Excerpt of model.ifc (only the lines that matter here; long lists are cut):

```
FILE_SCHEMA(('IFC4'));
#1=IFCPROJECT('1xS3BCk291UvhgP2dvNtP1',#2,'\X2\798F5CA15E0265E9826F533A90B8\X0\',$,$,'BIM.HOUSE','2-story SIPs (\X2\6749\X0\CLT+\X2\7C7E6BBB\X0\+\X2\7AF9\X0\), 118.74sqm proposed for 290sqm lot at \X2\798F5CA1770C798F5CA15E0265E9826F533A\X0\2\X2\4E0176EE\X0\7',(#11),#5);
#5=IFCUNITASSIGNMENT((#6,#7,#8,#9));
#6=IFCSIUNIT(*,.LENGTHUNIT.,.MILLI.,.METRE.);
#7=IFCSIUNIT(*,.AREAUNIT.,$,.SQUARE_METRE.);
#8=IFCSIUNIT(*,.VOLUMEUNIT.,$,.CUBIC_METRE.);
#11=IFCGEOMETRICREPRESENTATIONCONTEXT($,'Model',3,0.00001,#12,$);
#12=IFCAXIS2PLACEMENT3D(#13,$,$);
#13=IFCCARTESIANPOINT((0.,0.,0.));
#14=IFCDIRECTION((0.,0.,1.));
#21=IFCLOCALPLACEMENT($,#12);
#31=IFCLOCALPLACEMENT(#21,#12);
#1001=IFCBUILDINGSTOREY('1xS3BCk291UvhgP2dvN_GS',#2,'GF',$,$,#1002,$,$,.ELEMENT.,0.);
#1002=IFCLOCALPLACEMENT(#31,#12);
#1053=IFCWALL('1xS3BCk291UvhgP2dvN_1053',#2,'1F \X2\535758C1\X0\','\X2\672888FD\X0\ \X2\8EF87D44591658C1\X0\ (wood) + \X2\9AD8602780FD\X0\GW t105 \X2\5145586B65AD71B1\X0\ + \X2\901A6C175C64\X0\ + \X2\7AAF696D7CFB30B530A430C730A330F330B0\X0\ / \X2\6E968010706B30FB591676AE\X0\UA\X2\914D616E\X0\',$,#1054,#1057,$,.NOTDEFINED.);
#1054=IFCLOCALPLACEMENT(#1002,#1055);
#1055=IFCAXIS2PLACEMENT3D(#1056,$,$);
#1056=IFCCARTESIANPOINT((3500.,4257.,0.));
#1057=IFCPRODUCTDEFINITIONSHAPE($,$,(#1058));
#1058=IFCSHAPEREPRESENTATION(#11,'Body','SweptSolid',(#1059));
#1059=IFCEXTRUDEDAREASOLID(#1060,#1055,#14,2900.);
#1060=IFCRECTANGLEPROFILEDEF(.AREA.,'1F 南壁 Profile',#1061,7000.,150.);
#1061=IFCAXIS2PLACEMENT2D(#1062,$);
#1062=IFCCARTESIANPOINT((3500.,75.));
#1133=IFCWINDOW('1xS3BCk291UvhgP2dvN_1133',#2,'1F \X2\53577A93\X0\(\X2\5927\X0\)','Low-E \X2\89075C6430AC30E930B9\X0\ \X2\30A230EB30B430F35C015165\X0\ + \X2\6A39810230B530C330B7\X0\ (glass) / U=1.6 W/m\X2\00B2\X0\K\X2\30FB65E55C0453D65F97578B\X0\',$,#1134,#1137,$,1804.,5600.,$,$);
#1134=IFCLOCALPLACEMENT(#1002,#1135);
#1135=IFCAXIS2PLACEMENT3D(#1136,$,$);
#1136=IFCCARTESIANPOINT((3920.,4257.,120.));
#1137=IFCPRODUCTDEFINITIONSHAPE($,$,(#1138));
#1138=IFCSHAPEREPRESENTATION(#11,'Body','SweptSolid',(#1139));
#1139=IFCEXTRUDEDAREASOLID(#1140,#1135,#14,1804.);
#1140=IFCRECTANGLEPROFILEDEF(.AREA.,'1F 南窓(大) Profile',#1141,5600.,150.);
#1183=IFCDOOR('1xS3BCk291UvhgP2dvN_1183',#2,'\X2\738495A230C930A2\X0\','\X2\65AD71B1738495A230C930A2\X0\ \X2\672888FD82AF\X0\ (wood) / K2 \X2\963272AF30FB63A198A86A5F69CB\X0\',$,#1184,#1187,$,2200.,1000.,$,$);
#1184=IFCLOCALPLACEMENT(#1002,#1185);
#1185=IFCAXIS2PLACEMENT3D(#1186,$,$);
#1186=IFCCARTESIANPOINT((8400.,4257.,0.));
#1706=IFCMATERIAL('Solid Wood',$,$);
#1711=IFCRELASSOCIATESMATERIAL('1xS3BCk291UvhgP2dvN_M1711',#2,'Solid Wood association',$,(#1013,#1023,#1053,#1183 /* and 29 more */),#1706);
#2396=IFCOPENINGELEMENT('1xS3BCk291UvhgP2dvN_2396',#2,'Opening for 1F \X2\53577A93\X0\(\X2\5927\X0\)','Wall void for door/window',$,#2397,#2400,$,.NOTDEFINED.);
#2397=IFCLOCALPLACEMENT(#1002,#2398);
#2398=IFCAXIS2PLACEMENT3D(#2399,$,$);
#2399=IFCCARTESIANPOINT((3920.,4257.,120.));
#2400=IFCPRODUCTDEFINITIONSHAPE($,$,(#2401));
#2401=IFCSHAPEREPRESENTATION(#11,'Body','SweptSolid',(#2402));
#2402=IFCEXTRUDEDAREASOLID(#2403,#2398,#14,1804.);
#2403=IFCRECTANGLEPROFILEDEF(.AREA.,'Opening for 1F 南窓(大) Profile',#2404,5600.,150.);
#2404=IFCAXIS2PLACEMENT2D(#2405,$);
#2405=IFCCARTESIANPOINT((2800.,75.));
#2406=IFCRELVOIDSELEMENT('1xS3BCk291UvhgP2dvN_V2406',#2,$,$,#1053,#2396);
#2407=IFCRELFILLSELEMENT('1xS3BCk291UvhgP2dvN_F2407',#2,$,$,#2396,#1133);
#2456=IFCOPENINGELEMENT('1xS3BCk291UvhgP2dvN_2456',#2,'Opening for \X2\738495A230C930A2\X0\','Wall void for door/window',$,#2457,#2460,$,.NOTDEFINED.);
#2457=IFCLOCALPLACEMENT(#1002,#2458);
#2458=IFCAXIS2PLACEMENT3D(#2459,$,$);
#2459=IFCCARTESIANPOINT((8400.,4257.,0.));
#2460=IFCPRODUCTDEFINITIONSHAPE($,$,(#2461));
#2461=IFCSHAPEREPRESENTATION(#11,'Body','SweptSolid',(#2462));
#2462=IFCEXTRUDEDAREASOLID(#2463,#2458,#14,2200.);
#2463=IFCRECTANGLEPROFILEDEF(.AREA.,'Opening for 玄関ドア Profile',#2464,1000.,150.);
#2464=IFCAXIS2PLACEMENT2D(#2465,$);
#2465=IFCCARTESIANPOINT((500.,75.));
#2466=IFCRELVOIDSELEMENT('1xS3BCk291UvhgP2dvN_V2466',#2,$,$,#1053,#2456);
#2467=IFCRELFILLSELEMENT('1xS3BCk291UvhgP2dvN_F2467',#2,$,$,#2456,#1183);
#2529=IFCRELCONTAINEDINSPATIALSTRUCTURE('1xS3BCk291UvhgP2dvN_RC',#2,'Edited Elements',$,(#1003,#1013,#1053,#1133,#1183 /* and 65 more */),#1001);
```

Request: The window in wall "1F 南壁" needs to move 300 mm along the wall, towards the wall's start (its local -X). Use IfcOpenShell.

```python
import ifcopenshell
import ifcopenshell.api.geometry
import ifcopenshell.util.placement
import ifcopenshell.util.unit

model = ifcopenshell.open("model.ifc")
unit_scale = ifcopenshell.util.unit.calculate_unit_scale(model)

window = model.by_guid("1xS3BCk291UvhgP2dvN_1133")
opening = window.FillsVoids[0].RelatingOpeningElement
wall = opening.VoidsElements[0].RelatingBuildingElement

wall_matrix = ifcopenshell.util.placement.get_local_placement(wall.ObjectPlacement)
shift = wall_matrix[:3, 0] * -0.3 / unit_scale
before = ifcopenshell.util.placement.get_local_placement(window.ObjectPlacement)[:3, 3].copy()

# The window is not placed relative to its opening, so move both.
for product in (opening, window):
    matrix = ifcopenshell.util.placement.get_local_placement(product.ObjectPlacement)
    matrix[:3, 3] += shift
    ifcopenshell.api.geometry.edit_object_placement(model, product=product, matrix=matrix, is_si=False)

after = ifcopenshell.util.placement.get_local_placement(window.ObjectPlacement)[:3, 3]
print("window moved by", (after - before).round(3) + 0.0)

model.write("model_rev.ifc")
```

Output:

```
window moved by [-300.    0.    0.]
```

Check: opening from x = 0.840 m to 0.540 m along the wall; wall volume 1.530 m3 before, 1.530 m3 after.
